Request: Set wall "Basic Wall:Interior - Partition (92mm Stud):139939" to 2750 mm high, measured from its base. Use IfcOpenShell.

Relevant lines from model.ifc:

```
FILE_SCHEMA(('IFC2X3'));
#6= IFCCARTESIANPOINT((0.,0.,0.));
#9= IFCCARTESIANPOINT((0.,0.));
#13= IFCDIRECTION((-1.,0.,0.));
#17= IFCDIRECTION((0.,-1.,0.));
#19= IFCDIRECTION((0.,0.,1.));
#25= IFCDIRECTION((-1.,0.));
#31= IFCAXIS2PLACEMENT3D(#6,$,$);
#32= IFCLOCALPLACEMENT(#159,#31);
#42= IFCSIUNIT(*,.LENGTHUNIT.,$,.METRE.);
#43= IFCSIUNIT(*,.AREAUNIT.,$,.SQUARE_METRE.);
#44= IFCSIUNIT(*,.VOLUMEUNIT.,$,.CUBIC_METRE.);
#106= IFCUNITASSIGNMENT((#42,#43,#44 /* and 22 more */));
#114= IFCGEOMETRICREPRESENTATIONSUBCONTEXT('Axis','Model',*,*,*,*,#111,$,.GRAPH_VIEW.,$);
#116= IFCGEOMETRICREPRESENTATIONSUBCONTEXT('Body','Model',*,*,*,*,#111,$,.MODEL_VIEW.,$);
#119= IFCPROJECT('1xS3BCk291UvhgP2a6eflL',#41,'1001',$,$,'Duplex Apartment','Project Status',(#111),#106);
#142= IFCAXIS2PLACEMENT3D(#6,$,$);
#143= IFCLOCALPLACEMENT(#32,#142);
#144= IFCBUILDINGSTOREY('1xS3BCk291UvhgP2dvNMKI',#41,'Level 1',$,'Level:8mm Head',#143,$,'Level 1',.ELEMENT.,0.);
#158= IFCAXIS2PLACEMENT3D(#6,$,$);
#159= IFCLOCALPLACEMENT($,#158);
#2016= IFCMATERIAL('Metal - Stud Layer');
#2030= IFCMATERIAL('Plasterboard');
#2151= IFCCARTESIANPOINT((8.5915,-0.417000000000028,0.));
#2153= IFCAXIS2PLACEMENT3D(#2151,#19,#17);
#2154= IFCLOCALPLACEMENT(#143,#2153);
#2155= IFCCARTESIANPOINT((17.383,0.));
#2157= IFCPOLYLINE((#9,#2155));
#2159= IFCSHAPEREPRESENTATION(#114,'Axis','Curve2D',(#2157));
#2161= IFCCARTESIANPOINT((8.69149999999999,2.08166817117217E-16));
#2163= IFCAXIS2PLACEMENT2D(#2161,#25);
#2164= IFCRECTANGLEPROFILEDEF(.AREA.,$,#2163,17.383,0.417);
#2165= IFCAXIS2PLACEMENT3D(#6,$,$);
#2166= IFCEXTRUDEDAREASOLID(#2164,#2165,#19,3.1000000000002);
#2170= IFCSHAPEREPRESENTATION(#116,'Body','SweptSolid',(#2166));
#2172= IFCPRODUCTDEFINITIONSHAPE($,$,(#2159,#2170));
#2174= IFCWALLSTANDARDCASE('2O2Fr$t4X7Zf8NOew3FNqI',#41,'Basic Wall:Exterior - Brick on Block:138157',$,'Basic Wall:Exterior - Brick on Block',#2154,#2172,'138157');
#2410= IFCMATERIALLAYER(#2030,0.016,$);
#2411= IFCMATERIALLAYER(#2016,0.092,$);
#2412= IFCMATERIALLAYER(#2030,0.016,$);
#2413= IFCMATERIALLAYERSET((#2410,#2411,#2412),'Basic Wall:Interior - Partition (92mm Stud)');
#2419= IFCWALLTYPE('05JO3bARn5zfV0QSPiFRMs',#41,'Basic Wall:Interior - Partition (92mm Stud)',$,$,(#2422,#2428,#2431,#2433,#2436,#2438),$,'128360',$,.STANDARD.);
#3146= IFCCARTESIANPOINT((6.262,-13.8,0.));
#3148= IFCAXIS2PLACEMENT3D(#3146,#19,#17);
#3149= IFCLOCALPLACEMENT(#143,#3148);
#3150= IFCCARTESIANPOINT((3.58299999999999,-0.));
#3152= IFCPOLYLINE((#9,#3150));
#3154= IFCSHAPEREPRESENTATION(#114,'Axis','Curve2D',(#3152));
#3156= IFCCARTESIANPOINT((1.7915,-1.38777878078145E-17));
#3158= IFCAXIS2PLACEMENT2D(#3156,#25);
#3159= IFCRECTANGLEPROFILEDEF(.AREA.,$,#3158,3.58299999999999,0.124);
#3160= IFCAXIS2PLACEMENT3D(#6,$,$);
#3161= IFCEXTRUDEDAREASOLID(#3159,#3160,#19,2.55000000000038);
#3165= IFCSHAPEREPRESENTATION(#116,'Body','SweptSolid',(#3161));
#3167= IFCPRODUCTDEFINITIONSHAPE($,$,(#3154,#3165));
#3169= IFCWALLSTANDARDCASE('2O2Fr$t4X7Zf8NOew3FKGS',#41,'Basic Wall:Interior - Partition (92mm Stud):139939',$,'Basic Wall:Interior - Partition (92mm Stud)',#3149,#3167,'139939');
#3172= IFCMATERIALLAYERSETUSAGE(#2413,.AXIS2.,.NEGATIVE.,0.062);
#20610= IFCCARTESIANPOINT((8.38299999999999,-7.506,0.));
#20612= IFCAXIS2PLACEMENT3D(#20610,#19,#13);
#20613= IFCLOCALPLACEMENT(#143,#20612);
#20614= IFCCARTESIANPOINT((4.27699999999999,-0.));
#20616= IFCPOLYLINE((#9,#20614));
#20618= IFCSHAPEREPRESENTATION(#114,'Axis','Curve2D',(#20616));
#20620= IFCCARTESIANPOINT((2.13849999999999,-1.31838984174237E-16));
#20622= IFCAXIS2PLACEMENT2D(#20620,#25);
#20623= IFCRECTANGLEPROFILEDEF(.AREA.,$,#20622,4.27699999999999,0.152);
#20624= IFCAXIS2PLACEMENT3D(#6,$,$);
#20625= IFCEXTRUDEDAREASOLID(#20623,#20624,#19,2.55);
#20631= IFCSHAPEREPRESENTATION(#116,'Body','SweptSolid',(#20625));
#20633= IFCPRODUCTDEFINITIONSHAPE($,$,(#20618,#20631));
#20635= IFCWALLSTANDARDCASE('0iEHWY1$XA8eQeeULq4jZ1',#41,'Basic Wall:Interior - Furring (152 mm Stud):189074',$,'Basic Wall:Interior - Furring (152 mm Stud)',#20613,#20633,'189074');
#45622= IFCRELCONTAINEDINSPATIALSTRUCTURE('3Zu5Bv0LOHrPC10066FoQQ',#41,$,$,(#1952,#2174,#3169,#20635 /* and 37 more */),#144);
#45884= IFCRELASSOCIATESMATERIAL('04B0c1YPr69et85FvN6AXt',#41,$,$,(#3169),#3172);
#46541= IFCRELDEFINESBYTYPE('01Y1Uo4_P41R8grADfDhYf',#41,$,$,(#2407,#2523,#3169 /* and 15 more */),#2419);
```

```python
import ifcopenshell
import ifcopenshell.geom
import ifcopenshell.util.representation
import ifcopenshell.util.shape

model = ifcopenshell.open("model.ifc")
settings = ifcopenshell.geom.settings()


def volume(element):
    """Net volume in cubic metres, openings subtracted."""
    shape = ifcopenshell.geom.create_shape(settings, element)
    return ifcopenshell.util.shape.get_volume(shape.geometry)


wall = model.by_guid("2O2Fr$t4X7Zf8NOew3FKGS")
before = volume(wall)

body = ifcopenshell.util.representation.get_representation(wall, "Model", "Body")
solid = body.Items[0]
old_height = solid.Depth
solid.Depth = 2.75
after = volume(wall)

print(f"height {old_height:g} -> {solid.Depth:g}, volume {before:.3f} -> {after:.3f} m3")

model.write("model_v2.ifc")
```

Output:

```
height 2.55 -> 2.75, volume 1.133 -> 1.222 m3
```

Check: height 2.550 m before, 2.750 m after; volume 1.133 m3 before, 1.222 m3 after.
